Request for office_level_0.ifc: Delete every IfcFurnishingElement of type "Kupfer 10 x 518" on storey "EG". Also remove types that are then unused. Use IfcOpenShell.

First a look at what the model holds.

```python
import ifcopenshell
import ifcopenshell.util.element

model = ifcopenshell.open("office_level_0.ifc")
print(model.schema)
storey = next(s for s in model.by_type("IfcBuildingStorey") if s.Name == "EG")
furniture = [e for e in ifcopenshell.util.element.get_decomposition(storey) if e.is_a("IfcFurnishingElement")]
seen = {}
for e in furniture:
    element_type = ifcopenshell.util.element.get_type(e)
    name = element_type.Name if element_type not in (None, e) else None
    seen[name] = seen.get(name, 0) + 1
for name, count in sorted(seen.items(), key=str):
    print(count, "x", name)
```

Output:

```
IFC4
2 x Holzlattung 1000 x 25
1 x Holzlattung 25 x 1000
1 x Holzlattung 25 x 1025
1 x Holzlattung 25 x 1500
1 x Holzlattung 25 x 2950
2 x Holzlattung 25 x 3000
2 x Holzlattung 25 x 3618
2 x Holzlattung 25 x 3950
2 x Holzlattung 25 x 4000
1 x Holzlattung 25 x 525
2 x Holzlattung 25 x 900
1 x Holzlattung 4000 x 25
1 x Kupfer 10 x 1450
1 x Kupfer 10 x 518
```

```python
import ifcopenshell
import ifcopenshell.api.root
import ifcopenshell.util.element

model = ifcopenshell.open("office_level_0.ifc")

storey = next(s for s in model.by_type("IfcBuildingStorey") if s.Name == "EG")
furniture = [e for e in ifcopenshell.util.element.get_decomposition(storey) if e.is_a("IfcFurnishingElement")]
targets = [e for e in furniture if (t := ifcopenshell.util.element.get_type(e)) not in (None, e) and t.Name == "Kupfer 10 x 518"]
types = {ifcopenshell.util.element.get_type(e) for e in targets} - {None, *targets}

for e in targets:
    ifcopenshell.api.root.remove_product(model, product=e)
print(len(targets), "removed")

unused = [t for t in types if not ifcopenshell.util.element.get_types(t)]
for t in unused:
    ifcopenshell.api.root.remove_product(model, product=t)
print(len(unused), "unused types removed")

model.write("office_level_0_edited.ifc")
```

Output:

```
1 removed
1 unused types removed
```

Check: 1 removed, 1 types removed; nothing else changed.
